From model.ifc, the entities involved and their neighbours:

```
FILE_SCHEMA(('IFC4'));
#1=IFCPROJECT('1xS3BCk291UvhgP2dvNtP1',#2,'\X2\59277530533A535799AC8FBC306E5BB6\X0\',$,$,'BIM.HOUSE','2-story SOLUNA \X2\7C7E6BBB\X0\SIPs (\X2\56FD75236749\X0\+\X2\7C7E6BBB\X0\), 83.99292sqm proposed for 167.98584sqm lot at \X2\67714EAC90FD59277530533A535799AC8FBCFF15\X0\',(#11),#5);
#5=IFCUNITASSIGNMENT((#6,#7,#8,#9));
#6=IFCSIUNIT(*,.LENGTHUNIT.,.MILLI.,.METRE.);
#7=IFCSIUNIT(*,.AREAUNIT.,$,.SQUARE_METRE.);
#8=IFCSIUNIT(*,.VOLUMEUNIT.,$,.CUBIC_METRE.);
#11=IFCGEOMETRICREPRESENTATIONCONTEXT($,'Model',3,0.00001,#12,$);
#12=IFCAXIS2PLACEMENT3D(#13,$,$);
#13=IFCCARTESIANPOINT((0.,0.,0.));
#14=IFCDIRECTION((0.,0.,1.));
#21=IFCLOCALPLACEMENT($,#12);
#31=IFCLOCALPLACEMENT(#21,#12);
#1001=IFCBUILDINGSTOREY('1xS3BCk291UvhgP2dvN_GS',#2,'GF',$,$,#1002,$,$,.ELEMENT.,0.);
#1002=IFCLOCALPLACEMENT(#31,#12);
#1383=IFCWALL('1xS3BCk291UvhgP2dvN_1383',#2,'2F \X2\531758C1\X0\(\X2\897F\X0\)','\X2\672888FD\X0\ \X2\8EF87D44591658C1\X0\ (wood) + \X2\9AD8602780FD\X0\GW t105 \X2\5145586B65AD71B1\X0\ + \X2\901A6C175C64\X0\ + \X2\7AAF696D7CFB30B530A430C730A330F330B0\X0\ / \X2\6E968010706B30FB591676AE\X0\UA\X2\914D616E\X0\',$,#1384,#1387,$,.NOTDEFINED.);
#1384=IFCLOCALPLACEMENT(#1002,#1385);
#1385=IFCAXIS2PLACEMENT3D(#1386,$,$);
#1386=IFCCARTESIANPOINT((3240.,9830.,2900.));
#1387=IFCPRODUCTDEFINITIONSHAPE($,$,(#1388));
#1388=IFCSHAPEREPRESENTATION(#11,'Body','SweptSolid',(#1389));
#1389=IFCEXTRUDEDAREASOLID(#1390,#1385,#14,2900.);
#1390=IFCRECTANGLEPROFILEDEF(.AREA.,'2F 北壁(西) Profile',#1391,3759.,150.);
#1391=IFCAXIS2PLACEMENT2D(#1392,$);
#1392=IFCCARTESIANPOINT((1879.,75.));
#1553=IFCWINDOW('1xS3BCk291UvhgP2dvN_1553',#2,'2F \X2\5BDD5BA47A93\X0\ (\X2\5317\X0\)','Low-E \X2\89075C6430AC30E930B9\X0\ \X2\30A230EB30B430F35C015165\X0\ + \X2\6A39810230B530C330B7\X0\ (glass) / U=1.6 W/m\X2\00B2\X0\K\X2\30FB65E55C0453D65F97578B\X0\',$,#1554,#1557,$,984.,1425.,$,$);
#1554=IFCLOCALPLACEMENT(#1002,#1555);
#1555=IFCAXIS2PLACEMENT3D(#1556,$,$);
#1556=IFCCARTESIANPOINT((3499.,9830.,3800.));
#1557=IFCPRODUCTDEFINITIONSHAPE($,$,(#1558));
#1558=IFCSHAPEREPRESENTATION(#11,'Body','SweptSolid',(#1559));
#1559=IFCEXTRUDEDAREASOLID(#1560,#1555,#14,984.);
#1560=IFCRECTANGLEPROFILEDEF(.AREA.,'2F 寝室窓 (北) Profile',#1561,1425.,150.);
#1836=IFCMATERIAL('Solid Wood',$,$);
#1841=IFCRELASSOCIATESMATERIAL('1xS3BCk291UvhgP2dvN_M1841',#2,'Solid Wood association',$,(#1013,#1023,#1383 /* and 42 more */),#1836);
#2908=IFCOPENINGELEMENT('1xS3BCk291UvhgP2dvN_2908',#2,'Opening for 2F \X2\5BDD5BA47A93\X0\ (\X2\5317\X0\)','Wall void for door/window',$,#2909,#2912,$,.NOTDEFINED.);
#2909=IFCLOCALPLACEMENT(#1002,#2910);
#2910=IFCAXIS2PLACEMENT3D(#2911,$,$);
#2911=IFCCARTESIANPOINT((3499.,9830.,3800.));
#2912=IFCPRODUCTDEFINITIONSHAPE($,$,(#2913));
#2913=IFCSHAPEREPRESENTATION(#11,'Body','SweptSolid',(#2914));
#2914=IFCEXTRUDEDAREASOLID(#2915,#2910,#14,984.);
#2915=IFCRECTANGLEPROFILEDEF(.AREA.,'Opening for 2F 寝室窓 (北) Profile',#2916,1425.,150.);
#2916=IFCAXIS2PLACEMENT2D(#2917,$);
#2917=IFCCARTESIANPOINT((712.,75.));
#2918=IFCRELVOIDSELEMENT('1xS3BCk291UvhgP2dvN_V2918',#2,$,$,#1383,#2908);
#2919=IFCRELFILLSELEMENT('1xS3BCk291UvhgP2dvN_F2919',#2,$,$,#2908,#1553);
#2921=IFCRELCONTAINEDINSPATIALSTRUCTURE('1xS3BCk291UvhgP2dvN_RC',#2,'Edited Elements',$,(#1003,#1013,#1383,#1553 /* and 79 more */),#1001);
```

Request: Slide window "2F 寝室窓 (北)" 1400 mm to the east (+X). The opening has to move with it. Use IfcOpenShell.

```python
import ifcopenshell
import ifcopenshell.api.geometry
import ifcopenshell.util.placement

model = ifcopenshell.open("model.ifc")

window = model.by_guid("1xS3BCk291UvhgP2dvN_1553")
opening = window.FillsVoids[0].RelatingOpeningElement
wall = opening.VoidsElements[0].RelatingBuildingElement

wall_matrix = ifcopenshell.util.placement.get_local_placement(wall.ObjectPlacement)
shift = wall_matrix[:3, 0] * 1400.0
before = ifcopenshell.util.placement.get_local_placement(window.ObjectPlacement)[:3, 3].copy()

# The window is not placed relative to its opening, so move both.
for product in (opening, window):
    matrix = ifcopenshell.util.placement.get_local_placement(product.ObjectPlacement)
    matrix[:3, 3] += shift
    ifcopenshell.api.geometry.edit_object_placement(model, product=product, matrix=matrix, is_si=False)

after = ifcopenshell.util.placement.get_local_placement(window.ObjectPlacement)[:3, 3]
print("window moved by", (after - before).round(3) + 0.0)

model.write("model_updated.ifc")
```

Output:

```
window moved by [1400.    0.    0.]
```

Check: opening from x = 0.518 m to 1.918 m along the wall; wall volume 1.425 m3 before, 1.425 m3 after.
